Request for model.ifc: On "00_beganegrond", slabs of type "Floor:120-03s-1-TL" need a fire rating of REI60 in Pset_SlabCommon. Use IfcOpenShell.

First a look at what the model holds.

```python
import ifcopenshell
import ifcopenshell.util.element

model = ifcopenshell.open("model.ifc")
print(model.schema)
storey = next(s for s in model.by_type("IfcBuildingStorey") if s.Name == "00_beganegrond")
slabs = [e for e in ifcopenshell.util.element.get_decomposition(storey) if e.is_a("IfcSlab")]
seen = {}
for e in slabs:
    element_type = ifcopenshell.util.element.get_type(e)
    key = (element_type.Name if element_type != e and element_type else None, ifcopenshell.util.element.get_pset(e, "Pset_SlabCommon", "FireRating"))
    seen[key] = seen.get(key, 0) + 1
for (name, value), count in sorted(seen.items(), key=str):
    print(count, "x", name, "|", value)
```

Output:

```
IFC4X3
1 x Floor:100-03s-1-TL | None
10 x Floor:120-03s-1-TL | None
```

```python
import ifcopenshell
import ifcopenshell.api.pset
import ifcopenshell.util.element

model = ifcopenshell.open("model.ifc")

storey = next(s for s in model.by_type("IfcBuildingStorey") if s.Name == "00_beganegrond")
slabs = [e for e in ifcopenshell.util.element.get_decomposition(storey) if e.is_a("IfcSlab")]

count = 0
for e in slabs:
    element_type = ifcopenshell.util.element.get_type(e)
    if element_type in (None, e) or element_type.Name != "Floor:120-03s-1-TL":
        continue
    # add_pset returns the element's existing set when there is one.
    pset = ifcopenshell.api.pset.add_pset(model, product=e, name="Pset_SlabCommon")
    ifcopenshell.api.pset.edit_pset(model, pset=pset, properties={"FireRating": "REI60"})
    count += 1

print(count, "slabs updated")

model.write("model_v2.ifc")
```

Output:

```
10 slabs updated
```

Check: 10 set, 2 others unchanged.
